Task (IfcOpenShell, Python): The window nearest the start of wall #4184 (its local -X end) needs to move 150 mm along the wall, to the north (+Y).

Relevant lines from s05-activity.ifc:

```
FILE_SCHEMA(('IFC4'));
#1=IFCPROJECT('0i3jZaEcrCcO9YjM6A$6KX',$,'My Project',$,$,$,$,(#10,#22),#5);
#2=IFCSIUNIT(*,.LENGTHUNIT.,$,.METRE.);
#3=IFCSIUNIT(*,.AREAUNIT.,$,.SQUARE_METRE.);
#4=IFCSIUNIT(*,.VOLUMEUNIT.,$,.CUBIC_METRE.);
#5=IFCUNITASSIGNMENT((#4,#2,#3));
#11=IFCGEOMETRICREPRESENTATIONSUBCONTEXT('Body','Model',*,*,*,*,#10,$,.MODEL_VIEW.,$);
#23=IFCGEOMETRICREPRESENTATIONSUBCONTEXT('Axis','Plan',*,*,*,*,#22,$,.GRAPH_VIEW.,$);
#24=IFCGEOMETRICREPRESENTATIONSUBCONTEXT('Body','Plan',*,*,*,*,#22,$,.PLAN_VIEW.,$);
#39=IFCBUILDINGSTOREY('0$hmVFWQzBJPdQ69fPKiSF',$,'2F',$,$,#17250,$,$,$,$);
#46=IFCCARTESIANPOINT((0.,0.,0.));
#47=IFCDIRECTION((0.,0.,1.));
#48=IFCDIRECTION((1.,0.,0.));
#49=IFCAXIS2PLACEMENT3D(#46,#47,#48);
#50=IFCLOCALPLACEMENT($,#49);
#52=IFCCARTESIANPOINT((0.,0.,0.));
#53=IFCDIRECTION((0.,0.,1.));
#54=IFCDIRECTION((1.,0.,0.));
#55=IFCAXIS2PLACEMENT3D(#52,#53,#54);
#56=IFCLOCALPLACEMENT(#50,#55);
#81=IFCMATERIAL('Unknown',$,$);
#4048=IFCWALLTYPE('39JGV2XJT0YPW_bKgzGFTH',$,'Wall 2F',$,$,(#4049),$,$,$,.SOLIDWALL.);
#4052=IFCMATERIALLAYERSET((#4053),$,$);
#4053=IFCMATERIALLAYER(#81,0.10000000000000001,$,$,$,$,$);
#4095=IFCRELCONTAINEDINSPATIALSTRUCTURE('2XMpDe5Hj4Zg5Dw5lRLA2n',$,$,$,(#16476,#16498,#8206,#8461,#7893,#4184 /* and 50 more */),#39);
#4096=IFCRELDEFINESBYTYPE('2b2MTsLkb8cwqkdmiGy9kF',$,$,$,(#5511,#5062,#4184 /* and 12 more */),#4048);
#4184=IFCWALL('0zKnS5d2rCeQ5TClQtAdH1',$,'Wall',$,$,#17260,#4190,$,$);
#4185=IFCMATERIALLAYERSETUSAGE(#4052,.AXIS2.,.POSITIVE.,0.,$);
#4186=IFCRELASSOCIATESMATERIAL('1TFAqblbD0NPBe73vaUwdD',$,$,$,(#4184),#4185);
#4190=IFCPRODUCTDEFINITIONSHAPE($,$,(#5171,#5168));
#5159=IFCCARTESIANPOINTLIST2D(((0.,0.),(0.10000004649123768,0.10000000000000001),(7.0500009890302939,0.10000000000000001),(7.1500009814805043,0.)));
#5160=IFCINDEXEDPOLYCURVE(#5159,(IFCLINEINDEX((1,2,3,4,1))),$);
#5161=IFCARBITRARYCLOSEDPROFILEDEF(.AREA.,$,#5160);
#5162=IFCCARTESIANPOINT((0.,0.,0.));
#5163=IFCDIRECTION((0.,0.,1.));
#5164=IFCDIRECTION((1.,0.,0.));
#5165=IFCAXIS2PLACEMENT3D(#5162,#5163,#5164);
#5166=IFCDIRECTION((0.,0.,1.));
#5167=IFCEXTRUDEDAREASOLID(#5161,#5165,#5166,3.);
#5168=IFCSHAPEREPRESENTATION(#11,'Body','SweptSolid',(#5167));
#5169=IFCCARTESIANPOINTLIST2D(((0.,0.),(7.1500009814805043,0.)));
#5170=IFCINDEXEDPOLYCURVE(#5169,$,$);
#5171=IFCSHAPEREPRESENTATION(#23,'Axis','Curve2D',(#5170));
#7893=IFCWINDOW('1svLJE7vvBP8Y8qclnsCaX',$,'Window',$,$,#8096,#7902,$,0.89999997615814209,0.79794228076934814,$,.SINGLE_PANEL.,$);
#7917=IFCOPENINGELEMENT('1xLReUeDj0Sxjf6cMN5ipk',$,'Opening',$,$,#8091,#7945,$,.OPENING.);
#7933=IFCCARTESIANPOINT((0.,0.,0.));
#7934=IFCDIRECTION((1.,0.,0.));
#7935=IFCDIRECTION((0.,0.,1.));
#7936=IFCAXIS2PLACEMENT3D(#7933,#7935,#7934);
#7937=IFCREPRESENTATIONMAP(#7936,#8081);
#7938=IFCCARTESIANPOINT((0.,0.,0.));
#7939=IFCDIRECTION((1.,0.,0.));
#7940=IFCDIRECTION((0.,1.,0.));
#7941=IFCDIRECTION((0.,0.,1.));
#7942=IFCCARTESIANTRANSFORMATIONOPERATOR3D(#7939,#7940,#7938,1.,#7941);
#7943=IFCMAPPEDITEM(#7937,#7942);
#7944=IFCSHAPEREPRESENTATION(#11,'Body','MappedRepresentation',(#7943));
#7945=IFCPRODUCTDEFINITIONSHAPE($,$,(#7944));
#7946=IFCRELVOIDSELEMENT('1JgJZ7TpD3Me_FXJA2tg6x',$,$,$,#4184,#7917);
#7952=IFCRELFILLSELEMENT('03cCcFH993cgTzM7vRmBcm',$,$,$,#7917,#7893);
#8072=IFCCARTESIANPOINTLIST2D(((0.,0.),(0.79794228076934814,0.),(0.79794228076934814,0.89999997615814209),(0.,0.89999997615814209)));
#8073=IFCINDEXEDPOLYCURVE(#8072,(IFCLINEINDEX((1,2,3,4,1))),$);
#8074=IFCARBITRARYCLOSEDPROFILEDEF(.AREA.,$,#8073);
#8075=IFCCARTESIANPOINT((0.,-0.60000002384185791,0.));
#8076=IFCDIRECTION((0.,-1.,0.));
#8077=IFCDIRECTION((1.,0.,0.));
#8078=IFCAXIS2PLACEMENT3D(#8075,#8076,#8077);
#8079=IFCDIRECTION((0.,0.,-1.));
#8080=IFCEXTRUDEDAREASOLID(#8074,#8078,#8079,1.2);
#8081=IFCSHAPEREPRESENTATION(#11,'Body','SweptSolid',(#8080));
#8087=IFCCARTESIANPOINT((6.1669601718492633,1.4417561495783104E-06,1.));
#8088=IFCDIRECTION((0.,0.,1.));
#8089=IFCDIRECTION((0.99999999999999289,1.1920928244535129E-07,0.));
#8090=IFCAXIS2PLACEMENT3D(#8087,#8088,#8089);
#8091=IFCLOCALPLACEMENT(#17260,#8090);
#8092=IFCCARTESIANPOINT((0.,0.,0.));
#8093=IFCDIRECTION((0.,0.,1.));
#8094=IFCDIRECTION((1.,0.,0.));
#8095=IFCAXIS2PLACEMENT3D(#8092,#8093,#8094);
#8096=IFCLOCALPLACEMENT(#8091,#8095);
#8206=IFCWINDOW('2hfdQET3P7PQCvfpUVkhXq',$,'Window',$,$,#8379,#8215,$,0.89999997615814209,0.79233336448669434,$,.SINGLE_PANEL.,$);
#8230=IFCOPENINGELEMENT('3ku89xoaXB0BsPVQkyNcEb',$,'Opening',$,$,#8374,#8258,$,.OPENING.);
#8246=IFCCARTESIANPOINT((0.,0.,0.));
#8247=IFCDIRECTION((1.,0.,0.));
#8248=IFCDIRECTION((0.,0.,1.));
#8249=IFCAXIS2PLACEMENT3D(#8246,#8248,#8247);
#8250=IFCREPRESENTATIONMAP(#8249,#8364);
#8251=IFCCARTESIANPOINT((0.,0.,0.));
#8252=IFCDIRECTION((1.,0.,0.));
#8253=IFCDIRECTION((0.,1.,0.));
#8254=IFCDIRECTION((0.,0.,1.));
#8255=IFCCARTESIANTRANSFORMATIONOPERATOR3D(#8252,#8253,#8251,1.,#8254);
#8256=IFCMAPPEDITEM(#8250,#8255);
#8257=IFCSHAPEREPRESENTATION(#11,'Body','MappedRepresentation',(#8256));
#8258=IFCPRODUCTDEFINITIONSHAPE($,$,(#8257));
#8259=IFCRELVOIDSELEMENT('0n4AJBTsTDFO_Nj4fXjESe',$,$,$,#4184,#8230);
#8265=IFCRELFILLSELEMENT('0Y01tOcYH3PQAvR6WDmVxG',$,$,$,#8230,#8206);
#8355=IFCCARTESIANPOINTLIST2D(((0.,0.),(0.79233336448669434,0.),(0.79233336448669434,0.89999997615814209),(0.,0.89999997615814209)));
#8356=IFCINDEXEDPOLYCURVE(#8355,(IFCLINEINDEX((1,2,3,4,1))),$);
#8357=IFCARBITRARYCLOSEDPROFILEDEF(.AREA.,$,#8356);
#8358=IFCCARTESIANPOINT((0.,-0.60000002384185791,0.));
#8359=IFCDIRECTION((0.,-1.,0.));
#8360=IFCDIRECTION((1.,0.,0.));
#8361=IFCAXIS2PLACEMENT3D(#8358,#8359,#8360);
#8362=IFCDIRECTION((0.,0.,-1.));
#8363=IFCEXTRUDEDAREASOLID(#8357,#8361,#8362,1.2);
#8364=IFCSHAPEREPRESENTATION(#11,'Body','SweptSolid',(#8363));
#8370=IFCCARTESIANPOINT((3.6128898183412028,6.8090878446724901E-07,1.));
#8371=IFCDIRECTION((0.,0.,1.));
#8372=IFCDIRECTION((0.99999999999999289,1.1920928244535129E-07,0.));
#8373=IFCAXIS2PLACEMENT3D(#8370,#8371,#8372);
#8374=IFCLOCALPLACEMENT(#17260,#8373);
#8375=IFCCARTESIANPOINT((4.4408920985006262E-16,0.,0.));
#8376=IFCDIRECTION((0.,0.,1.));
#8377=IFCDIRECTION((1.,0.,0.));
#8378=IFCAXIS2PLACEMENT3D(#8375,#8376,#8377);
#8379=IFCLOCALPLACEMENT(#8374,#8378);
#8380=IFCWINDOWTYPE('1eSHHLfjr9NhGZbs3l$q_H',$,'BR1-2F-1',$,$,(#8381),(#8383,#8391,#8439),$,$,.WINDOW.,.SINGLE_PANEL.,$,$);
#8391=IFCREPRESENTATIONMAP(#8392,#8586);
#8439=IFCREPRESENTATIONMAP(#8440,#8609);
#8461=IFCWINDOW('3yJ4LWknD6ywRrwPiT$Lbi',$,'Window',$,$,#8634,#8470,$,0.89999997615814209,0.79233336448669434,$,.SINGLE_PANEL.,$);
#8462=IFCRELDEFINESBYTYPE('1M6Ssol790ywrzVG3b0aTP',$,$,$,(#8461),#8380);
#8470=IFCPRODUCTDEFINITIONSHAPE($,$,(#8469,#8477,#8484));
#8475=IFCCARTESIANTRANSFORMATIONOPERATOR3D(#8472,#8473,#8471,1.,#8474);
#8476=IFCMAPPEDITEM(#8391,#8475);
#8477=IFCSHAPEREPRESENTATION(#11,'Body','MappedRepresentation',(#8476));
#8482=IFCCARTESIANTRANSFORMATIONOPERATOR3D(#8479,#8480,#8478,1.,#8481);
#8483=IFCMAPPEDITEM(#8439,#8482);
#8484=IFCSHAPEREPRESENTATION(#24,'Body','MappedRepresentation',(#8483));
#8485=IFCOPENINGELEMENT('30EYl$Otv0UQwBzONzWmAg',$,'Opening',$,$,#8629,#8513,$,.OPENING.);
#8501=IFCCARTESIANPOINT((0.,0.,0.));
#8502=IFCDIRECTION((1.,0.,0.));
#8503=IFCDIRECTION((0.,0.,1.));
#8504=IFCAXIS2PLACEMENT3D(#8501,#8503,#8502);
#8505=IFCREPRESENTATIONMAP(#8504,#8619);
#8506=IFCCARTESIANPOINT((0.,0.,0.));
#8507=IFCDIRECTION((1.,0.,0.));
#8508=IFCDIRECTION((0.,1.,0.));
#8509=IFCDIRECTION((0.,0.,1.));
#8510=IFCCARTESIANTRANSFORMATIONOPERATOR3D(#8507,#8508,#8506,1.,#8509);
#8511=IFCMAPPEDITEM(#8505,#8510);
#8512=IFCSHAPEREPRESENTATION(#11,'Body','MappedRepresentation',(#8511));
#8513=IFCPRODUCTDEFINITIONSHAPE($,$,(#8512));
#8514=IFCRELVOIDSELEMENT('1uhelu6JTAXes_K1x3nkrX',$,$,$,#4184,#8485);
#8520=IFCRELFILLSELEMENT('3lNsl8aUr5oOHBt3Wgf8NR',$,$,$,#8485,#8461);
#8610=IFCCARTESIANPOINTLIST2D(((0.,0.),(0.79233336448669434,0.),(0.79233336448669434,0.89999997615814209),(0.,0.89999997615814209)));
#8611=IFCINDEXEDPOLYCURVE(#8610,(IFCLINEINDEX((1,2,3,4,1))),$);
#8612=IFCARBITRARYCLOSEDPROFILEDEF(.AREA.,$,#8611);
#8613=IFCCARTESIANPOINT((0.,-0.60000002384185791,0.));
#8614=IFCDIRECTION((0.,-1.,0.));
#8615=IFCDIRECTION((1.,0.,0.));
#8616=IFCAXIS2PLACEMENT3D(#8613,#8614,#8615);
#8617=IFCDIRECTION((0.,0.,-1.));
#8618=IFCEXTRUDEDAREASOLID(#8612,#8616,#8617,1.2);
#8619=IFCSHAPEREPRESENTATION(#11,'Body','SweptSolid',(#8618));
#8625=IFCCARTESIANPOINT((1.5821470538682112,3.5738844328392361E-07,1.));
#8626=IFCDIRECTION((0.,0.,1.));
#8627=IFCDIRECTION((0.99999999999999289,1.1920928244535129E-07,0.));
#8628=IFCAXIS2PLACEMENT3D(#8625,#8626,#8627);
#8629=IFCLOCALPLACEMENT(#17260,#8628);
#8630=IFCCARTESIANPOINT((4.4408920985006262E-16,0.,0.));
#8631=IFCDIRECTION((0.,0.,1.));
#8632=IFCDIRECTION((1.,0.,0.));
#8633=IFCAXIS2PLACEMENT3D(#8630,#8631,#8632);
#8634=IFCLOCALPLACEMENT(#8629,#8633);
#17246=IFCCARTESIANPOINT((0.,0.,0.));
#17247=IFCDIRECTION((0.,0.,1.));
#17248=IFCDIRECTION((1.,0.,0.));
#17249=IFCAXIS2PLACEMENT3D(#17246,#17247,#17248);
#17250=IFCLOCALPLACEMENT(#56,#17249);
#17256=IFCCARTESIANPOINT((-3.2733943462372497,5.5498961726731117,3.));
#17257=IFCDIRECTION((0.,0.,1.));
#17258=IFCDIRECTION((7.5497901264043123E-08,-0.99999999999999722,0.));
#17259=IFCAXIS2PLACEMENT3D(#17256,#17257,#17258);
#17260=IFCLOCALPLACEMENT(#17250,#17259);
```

```python
import ifcopenshell
import ifcopenshell.api.geometry
import ifcopenshell.util.placement
import ifcopenshell.util.unit

model = ifcopenshell.open("s05-activity.ifc")
unit_scale = ifcopenshell.util.unit.calculate_unit_scale(model)

window = model.by_guid("3yJ4LWknD6ywRrwPiT$Lbi")
opening = window.FillsVoids[0].RelatingOpeningElement
wall = opening.VoidsElements[0].RelatingBuildingElement

wall_matrix = ifcopenshell.util.placement.get_local_placement(wall.ObjectPlacement)
shift = wall_matrix[:3, 0] * -0.15 / unit_scale
before = ifcopenshell.util.placement.get_local_placement(window.ObjectPlacement)[:3, 3].copy()

# The window is placed relative to its opening, so it follows when the opening moves.
matrix = ifcopenshell.util.placement.get_local_placement(opening.ObjectPlacement)
matrix[:3, 3] += shift
ifcopenshell.api.geometry.edit_object_placement(
    model, product=opening, matrix=matrix, is_si=False, should_transform_children=True
)

after = ifcopenshell.util.placement.get_local_placement(window.ObjectPlacement)[:3, 3]
print("window moved by", (after - before).round(3) + 0.0)

model.write("s05-activity_edited.ifc")
```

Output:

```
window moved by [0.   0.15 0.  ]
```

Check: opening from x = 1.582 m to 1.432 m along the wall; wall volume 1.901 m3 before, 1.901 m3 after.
